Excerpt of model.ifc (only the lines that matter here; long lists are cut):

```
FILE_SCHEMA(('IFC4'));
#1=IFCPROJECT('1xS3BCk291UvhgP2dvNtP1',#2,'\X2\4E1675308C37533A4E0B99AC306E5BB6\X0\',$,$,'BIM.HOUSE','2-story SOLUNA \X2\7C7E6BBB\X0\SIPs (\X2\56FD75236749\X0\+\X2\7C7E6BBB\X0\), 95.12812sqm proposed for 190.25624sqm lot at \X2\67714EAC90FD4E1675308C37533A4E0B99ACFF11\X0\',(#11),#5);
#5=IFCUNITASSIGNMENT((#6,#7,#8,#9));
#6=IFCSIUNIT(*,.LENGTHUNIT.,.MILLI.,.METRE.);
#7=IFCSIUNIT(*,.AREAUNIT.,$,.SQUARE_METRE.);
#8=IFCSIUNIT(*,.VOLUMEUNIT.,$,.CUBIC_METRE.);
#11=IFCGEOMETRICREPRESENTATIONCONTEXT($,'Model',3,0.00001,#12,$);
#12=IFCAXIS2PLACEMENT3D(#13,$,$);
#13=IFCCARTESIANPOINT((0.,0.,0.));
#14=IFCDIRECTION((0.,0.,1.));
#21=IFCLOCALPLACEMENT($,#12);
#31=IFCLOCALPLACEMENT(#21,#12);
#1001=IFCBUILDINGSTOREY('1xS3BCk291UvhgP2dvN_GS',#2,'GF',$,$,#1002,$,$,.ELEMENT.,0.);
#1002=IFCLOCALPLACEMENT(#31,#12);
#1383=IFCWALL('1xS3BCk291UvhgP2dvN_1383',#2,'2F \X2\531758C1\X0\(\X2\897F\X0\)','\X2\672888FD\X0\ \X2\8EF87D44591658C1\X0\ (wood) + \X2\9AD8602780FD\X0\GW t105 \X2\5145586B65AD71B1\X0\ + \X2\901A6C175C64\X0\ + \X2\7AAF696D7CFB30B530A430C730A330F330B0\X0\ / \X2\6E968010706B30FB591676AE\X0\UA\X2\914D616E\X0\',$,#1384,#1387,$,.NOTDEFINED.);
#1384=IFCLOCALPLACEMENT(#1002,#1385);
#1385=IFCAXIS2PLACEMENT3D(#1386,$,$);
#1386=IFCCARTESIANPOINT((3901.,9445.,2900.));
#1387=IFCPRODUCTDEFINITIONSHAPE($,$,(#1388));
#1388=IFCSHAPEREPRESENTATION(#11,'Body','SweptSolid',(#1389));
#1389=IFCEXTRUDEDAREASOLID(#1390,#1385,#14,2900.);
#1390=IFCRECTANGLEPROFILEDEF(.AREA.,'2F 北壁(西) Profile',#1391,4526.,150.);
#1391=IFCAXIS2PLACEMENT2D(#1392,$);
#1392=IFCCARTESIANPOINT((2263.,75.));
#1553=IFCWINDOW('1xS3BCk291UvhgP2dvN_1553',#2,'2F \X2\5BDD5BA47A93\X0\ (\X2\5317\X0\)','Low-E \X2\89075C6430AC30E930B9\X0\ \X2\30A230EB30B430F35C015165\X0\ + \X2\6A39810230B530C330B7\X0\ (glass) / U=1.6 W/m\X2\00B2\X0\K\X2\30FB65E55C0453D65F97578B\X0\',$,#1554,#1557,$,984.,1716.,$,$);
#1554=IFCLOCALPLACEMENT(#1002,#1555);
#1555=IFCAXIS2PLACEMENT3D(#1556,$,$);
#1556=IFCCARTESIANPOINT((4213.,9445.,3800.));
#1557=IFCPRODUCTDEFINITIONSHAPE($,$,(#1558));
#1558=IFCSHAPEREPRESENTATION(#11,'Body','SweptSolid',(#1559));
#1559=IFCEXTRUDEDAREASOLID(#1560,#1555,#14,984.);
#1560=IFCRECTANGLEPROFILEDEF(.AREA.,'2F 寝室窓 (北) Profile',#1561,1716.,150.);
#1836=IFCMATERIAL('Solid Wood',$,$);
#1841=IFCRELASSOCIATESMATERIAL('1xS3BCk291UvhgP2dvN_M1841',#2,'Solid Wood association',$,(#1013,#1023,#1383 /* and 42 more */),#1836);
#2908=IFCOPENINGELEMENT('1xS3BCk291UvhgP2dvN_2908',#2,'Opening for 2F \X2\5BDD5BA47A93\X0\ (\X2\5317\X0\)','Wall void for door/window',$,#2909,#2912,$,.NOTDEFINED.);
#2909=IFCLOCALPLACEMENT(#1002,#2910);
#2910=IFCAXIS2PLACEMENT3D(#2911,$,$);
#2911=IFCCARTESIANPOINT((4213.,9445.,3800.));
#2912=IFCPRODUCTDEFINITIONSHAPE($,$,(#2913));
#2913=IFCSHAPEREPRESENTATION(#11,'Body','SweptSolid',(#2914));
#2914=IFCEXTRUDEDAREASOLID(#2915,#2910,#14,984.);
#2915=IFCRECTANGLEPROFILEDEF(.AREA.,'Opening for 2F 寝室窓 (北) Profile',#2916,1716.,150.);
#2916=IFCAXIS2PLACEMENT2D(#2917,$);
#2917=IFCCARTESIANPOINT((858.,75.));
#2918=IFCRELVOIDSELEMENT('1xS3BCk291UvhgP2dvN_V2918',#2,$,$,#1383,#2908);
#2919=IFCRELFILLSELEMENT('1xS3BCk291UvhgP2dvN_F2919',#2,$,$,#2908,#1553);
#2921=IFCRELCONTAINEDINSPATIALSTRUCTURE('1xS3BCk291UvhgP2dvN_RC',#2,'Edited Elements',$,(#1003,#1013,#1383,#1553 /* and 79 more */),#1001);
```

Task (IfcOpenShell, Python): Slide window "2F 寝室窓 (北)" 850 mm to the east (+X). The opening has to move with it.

```python
import ifcopenshell
import ifcopenshell.api.geometry
import ifcopenshell.util.placement

model = ifcopenshell.open("model.ifc")

window = model.by_guid("1xS3BCk291UvhgP2dvN_1553")
opening = window.FillsVoids[0].RelatingOpeningElement
wall = opening.VoidsElements[0].RelatingBuildingElement

wall_matrix = ifcopenshell.util.placement.get_local_placement(wall.ObjectPlacement)
shift = wall_matrix[:3, 0] * 850.0
before = ifcopenshell.util.placement.get_local_placement(window.ObjectPlacement)[:3, 3].copy()

# The window is not placed relative to its opening, so move both.
for product in (opening, window):
    matrix = ifcopenshell.util.placement.get_local_placement(product.ObjectPlacement)
    matrix[:3, 3] += shift
    ifcopenshell.api.geometry.edit_object_placement(model, product=product, matrix=matrix, is_si=False)

after = ifcopenshell.util.placement.get_local_placement(window.ObjectPlacement)[:3, 3]
print("window moved by", (after - before).round(3) + 0.0)

model.write("model_rev.ifc")
```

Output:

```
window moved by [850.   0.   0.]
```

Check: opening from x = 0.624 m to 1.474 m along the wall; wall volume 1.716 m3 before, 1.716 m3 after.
